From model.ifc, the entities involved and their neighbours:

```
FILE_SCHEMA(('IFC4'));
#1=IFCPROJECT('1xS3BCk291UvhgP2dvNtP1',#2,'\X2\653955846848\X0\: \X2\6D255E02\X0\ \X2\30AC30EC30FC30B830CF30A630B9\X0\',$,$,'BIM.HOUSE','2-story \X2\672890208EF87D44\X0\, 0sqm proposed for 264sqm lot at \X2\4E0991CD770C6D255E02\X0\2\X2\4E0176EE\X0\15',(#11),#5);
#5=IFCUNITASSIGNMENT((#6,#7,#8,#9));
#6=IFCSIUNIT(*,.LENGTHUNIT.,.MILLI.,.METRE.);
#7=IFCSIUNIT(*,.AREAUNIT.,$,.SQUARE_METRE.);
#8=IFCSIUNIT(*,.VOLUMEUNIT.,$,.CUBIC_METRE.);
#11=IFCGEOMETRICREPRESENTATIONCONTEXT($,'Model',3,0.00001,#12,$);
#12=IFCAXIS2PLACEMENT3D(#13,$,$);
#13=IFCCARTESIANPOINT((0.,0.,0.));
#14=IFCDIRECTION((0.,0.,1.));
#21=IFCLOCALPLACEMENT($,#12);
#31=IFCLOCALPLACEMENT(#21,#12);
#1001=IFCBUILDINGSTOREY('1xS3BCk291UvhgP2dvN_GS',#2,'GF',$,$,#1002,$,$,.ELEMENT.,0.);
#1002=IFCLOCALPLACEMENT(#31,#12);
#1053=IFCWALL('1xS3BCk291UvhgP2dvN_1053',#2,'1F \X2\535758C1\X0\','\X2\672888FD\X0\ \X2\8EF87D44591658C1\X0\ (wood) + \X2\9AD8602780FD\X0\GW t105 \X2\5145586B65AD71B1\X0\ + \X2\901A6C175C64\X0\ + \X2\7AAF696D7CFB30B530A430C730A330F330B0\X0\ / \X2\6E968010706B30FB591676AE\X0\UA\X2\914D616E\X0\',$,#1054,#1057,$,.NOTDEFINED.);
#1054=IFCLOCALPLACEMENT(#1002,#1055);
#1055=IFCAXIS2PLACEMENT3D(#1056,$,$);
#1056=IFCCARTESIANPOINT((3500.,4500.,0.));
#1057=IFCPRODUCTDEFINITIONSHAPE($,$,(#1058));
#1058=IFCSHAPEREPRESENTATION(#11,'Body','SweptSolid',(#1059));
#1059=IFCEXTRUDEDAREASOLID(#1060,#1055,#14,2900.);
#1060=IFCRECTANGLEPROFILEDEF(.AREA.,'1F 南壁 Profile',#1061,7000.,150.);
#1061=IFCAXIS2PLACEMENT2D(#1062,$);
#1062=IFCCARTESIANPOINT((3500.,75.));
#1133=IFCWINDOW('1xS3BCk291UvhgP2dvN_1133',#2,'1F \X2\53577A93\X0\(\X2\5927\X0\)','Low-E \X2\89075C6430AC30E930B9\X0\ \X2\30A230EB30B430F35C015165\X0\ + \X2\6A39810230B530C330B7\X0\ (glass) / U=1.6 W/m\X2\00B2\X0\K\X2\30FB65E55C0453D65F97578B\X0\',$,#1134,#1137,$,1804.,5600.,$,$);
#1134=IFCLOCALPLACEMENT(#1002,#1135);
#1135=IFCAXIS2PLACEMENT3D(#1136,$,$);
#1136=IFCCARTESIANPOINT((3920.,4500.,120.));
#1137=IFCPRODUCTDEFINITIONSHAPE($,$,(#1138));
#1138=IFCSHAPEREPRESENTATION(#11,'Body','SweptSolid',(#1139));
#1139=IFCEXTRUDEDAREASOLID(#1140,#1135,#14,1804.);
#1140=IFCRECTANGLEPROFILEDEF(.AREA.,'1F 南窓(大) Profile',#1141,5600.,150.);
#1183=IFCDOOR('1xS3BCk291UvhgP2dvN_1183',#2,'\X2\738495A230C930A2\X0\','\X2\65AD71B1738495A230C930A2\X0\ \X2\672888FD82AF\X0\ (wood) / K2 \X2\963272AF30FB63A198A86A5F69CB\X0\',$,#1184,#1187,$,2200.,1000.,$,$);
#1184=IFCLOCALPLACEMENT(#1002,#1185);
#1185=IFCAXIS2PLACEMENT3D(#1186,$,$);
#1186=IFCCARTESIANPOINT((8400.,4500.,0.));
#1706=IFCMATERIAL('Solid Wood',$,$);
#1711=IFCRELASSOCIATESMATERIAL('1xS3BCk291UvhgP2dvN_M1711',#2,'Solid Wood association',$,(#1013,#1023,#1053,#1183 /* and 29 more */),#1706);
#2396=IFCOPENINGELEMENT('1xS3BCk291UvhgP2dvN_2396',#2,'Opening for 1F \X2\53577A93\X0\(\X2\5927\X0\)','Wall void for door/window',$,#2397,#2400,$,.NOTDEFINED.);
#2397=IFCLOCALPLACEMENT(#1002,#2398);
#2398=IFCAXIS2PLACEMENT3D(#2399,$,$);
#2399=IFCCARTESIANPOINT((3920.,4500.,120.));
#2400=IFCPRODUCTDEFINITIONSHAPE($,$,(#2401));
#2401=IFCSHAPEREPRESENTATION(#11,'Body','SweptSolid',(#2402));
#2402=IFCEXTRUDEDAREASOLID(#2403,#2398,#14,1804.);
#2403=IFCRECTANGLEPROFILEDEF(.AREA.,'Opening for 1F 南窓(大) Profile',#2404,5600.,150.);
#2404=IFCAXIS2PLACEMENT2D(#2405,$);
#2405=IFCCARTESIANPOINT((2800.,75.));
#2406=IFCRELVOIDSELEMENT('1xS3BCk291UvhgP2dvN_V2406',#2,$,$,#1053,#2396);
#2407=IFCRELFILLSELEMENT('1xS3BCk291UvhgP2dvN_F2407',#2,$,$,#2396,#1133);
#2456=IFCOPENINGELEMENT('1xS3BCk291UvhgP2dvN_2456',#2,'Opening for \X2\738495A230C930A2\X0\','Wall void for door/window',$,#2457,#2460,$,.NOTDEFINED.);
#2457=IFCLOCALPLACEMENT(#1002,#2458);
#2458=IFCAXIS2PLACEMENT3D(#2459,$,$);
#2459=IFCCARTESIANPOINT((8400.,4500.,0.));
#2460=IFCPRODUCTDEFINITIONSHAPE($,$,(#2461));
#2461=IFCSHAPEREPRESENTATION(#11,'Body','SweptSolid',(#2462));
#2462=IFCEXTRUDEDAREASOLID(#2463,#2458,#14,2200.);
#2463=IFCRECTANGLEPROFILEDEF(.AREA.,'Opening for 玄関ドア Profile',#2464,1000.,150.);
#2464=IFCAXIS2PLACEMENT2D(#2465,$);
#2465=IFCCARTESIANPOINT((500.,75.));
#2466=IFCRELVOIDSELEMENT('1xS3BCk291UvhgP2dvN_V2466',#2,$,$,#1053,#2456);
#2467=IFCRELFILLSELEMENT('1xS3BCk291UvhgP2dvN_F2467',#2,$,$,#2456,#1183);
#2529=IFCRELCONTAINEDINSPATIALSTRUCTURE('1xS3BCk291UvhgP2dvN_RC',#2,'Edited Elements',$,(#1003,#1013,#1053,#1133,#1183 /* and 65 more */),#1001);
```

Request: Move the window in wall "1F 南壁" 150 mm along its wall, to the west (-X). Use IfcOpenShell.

```python
import ifcopenshell
import ifcopenshell.api.geometry
import ifcopenshell.util.placement

model = ifcopenshell.open("model.ifc")

window = model.by_guid("1xS3BCk291UvhgP2dvN_1133")
opening = window.FillsVoids[0].RelatingOpeningElement
wall = opening.VoidsElements[0].RelatingBuildingElement

wall_matrix = ifcopenshell.util.placement.get_local_placement(wall.ObjectPlacement)
shift = wall_matrix[:3, 0] * -150.0
before = ifcopenshell.util.placement.get_local_placement(window.ObjectPlacement)[:3, 3].copy()

# The window is not placed relative to its opening, so move both.
for product in (opening, window):
    matrix = ifcopenshell.util.placement.get_local_placement(product.ObjectPlacement)
    matrix[:3, 3] += shift
    ifcopenshell.api.geometry.edit_object_placement(model, product=product, matrix=matrix, is_si=False)

after = ifcopenshell.util.placement.get_local_placement(window.ObjectPlacement)[:3, 3]
print("window moved by", (after - before).round(3) + 0.0)

model.write("model_updated.ifc")
```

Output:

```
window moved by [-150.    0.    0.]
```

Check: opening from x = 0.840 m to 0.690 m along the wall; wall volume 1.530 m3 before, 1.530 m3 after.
